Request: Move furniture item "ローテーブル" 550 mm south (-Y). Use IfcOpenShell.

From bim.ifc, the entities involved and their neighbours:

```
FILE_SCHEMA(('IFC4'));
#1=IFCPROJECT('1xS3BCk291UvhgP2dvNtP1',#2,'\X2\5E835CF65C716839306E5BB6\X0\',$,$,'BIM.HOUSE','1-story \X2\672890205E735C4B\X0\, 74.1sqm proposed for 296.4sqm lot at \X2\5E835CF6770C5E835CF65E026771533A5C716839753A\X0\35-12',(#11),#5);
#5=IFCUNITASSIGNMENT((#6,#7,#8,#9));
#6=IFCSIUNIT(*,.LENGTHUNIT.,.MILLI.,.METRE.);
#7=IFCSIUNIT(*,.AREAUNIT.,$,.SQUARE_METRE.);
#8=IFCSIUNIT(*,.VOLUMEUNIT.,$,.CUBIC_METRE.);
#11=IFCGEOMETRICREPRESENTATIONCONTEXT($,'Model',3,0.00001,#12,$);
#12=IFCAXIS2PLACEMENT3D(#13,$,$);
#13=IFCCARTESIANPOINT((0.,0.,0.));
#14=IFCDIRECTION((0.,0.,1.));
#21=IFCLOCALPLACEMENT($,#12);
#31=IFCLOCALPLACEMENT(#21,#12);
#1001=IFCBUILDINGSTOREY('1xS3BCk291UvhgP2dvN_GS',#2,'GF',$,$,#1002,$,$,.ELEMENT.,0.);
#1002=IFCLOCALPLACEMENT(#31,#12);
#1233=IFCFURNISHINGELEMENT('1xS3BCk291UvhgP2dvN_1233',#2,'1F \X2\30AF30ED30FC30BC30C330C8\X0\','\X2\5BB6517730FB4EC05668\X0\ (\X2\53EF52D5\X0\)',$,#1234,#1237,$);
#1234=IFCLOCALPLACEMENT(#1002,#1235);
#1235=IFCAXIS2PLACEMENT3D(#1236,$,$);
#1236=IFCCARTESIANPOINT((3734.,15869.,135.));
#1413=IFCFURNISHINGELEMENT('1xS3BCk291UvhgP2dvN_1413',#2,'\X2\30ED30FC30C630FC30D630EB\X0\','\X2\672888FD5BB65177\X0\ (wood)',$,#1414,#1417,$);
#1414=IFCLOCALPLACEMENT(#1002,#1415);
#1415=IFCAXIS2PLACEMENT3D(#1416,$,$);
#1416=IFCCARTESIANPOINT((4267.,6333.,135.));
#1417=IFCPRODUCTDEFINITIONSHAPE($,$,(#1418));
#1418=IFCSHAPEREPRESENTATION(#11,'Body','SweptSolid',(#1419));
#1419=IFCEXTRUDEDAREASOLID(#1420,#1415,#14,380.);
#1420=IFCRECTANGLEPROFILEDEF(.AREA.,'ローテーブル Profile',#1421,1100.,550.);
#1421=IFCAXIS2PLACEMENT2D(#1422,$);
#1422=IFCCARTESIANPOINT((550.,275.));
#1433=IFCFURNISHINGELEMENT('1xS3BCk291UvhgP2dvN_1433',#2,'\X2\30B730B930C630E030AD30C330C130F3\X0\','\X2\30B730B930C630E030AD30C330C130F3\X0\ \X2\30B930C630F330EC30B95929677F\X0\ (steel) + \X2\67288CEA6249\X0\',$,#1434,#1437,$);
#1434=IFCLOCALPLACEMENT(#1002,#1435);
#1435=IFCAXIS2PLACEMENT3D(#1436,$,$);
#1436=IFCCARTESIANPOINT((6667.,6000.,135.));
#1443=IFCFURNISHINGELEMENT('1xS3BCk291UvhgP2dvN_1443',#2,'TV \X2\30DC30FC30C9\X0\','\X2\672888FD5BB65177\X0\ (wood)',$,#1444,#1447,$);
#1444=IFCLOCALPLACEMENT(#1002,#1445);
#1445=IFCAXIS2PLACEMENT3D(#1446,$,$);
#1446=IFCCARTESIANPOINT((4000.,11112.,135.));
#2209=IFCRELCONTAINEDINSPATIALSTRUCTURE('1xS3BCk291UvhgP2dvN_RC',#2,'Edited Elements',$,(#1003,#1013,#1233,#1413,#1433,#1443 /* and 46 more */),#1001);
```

```python
import ifcopenshell
import ifcopenshell.api.geometry
import ifcopenshell.util.placement
import ifcopenshell.util.unit

model = ifcopenshell.open("bim.ifc")
unit_scale = ifcopenshell.util.unit.calculate_unit_scale(model)

item = model.by_guid("1xS3BCk291UvhgP2dvN_1413")
matrix = ifcopenshell.util.placement.get_local_placement(item.ObjectPlacement)
matrix[1, 3] -= 0.55 / unit_scale
ifcopenshell.api.geometry.edit_object_placement(model, product=item, matrix=matrix, is_si=False)

print(ifcopenshell.util.placement.get_local_placement(item.ObjectPlacement).round(3) + 0.0)

model.write("bim_v2.ifc")
```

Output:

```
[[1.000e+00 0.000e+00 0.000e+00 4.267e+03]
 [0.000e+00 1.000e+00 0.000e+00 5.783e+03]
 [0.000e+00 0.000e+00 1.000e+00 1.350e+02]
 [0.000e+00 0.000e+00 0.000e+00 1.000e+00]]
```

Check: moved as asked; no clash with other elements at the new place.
